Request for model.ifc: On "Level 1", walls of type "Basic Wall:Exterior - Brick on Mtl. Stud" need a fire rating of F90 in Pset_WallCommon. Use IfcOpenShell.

First a look at what the model holds.

```python
import ifcopenshell
import ifcopenshell.util.element

model = ifcopenshell.open("model.ifc")
print(model.schema)
storey = next(s for s in model.by_type("IfcBuildingStorey") if s.Name == "Level 1")
walls = [e for e in ifcopenshell.util.element.get_decomposition(storey) if e.is_a("IfcWall")]
seen = {}
for e in walls:
    element_type = ifcopenshell.util.element.get_type(e)
    key = (element_type.Name if element_type != e and element_type else None, ifcopenshell.util.element.get_pset(e, "Pset_WallCommon", "FireRating"))
    seen[key] = seen.get(key, 0) + 1
for (name, value), count in sorted(seen.items(), key=str):
    print(count, "x", name, "|", value)
```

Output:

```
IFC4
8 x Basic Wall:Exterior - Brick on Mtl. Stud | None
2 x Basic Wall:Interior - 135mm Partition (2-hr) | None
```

```python
import ifcopenshell
import ifcopenshell.api.pset
import ifcopenshell.util.element

model = ifcopenshell.open("model.ifc")

storey = next(s for s in model.by_type("IfcBuildingStorey") if s.Name == "Level 1")
walls = [e for e in ifcopenshell.util.element.get_decomposition(storey) if e.is_a("IfcWall")]

count = 0
for e in walls:
    element_type = ifcopenshell.util.element.get_type(e)
    if element_type in (None, e) or element_type.Name != "Basic Wall:Exterior - Brick on Mtl. Stud":
        continue
    # add_pset returns the element's existing set when there is one.
    pset = ifcopenshell.api.pset.add_pset(model, product=e, name="Pset_WallCommon")
    ifcopenshell.api.pset.edit_pset(model, pset=pset, properties={"FireRating": "F90"})
    count += 1

print(count, "walls updated")

model.write("model_updated.ifc")
```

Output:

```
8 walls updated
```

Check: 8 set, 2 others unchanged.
